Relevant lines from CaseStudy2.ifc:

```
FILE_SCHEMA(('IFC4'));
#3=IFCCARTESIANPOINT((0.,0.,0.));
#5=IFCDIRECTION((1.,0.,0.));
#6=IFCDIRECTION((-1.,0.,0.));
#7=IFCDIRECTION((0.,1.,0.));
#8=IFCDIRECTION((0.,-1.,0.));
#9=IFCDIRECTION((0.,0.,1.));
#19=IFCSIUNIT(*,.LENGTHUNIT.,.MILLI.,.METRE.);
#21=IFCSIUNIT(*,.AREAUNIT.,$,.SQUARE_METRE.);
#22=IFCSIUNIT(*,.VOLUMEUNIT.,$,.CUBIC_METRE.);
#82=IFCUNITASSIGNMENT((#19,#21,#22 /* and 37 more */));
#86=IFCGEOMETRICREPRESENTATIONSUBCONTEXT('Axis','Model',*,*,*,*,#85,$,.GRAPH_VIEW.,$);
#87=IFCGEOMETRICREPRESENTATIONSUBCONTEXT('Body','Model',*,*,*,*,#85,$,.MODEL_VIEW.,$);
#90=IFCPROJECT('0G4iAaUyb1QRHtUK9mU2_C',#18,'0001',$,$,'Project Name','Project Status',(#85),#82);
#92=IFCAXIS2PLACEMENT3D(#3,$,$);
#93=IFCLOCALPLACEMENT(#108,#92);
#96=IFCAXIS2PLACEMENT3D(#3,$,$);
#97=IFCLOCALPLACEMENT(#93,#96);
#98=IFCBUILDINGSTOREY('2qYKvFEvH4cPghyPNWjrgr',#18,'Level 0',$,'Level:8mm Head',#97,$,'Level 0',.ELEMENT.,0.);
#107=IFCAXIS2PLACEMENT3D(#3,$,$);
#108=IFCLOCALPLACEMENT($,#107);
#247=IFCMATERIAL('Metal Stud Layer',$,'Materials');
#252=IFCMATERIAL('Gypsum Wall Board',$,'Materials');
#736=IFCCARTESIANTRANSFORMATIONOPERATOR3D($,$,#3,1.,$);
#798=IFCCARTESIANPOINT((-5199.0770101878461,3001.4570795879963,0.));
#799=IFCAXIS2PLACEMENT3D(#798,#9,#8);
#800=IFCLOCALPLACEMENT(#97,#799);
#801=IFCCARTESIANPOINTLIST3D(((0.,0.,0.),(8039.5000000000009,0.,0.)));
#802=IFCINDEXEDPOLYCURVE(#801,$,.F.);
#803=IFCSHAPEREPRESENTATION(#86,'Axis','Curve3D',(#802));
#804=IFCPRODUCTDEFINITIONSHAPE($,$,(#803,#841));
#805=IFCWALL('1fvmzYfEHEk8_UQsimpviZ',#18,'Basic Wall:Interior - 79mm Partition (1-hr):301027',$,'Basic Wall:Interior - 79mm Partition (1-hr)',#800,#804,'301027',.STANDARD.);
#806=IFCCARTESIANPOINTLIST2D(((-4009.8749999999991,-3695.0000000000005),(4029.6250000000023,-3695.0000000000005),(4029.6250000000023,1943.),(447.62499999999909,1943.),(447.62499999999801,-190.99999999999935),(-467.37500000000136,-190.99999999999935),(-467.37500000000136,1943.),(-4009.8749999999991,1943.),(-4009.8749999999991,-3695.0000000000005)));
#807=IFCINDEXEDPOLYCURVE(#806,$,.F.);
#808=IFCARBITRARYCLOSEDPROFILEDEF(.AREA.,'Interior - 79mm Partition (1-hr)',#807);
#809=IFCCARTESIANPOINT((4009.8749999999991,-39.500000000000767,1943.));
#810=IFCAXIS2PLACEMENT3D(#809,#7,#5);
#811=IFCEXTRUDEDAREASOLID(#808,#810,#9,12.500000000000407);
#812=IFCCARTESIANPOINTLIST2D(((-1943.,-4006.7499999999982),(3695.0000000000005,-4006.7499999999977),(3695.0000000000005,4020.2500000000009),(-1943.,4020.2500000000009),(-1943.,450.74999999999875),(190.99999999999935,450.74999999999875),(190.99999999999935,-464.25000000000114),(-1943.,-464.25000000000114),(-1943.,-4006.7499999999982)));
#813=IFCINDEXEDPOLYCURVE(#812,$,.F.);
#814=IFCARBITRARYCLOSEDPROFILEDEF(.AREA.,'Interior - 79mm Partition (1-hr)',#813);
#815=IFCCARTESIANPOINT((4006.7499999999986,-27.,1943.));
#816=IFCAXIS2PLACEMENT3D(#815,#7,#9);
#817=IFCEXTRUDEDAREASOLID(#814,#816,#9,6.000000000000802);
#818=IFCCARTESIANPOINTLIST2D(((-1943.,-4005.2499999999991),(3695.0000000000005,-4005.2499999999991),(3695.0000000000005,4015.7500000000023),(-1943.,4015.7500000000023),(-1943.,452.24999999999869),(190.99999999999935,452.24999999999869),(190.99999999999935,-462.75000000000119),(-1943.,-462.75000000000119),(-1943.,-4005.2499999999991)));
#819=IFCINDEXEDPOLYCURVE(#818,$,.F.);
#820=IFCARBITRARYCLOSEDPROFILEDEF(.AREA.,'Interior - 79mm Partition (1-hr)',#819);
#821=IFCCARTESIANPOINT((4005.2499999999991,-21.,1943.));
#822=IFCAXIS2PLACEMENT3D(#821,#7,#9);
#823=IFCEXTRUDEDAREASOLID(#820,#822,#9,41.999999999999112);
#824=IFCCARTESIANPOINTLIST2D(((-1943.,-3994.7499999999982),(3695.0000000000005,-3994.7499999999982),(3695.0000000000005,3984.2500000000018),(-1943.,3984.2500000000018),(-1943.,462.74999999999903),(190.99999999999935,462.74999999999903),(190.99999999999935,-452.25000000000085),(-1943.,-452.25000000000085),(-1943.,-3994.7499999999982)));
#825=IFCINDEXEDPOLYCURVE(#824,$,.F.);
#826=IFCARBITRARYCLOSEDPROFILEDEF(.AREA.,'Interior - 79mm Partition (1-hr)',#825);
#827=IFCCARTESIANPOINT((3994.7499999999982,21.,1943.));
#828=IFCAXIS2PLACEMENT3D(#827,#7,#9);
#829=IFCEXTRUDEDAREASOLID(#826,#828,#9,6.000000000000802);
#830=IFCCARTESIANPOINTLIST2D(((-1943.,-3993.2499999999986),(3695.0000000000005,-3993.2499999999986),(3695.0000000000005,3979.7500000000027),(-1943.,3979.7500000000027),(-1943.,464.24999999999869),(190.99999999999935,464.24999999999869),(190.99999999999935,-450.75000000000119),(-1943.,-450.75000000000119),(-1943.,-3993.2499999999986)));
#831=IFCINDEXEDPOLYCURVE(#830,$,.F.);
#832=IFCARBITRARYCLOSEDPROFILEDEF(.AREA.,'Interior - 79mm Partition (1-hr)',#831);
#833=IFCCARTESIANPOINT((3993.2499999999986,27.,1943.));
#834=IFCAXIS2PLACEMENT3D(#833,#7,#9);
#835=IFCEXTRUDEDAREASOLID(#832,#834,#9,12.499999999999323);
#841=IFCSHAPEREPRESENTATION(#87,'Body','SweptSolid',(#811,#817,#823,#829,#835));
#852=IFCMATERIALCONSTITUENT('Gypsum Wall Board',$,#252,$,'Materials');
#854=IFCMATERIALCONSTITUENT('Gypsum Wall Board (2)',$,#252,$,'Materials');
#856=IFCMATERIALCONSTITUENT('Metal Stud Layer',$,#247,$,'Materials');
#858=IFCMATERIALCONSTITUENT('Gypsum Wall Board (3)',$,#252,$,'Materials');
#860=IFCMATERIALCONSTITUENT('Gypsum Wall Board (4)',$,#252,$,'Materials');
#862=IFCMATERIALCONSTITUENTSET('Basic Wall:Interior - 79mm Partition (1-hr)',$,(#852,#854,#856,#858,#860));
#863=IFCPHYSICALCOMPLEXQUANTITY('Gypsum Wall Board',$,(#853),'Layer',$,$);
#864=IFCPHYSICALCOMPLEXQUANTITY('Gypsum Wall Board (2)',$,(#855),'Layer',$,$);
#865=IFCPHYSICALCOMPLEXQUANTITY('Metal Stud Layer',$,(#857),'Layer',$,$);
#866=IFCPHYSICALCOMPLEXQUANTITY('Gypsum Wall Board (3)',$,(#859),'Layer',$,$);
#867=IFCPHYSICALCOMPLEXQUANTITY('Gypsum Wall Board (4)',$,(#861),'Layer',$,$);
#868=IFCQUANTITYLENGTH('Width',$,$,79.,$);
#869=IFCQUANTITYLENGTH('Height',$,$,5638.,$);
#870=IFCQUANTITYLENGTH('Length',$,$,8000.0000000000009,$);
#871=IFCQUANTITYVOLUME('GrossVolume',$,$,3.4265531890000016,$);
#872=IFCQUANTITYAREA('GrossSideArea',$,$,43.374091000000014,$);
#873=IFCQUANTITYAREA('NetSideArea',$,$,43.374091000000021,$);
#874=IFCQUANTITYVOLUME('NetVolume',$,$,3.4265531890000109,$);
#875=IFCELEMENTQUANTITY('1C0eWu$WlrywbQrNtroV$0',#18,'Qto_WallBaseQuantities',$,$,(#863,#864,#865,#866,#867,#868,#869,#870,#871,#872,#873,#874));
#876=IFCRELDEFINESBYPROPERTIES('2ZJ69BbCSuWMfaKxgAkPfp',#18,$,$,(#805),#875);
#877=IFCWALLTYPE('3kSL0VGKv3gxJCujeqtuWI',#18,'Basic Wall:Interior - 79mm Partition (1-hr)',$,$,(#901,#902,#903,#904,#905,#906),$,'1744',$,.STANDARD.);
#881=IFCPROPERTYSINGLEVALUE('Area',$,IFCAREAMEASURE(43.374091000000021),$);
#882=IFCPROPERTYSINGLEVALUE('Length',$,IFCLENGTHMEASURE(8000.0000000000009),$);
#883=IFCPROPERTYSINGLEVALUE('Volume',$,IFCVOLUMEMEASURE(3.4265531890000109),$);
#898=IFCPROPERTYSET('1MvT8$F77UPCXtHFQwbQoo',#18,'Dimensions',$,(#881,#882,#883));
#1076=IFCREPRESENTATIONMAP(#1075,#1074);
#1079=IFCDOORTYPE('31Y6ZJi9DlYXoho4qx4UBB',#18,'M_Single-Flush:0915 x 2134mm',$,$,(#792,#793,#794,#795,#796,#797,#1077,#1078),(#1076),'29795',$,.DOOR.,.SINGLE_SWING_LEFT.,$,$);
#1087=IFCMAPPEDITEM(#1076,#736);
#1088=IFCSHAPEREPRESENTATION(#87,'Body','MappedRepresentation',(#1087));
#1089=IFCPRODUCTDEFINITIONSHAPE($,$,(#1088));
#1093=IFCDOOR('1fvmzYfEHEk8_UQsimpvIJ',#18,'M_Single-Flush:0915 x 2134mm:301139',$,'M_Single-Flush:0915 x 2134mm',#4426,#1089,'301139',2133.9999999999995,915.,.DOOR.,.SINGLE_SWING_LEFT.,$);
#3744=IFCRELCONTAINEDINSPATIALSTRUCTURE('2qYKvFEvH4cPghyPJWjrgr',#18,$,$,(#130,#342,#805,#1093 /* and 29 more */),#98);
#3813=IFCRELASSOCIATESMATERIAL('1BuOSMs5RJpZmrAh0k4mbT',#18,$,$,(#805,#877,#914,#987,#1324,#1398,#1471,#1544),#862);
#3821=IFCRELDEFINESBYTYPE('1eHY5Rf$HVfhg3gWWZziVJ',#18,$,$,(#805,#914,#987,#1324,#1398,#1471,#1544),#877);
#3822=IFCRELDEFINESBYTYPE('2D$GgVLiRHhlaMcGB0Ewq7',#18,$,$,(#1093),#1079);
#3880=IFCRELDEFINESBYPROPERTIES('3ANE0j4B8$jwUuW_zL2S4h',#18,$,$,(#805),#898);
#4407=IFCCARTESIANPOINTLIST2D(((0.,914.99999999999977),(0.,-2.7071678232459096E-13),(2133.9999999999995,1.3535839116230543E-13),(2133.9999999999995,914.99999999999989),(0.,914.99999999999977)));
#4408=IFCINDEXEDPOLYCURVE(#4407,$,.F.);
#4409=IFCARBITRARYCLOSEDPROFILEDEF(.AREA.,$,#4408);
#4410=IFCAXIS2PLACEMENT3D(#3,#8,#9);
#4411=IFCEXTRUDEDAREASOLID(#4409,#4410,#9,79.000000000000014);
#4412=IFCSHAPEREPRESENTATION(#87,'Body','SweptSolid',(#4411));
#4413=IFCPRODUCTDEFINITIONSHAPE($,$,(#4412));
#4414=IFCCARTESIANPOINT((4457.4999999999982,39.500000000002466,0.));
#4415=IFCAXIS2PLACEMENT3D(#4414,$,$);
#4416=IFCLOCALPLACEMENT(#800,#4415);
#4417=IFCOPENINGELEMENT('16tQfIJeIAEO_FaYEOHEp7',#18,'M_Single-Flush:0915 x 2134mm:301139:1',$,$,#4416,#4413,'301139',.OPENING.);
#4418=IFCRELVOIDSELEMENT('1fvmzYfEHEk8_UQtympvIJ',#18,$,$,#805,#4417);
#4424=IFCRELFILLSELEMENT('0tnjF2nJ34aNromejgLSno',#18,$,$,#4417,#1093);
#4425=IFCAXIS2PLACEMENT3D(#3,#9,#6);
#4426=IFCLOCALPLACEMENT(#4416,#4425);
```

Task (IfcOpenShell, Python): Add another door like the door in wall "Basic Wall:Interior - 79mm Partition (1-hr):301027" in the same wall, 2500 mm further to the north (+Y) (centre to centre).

```python
import ifcopenshell
import ifcopenshell.api.feature
import ifcopenshell.api.geometry
import ifcopenshell.api.pset
import ifcopenshell.api.root
import ifcopenshell.geom
import ifcopenshell.util.element
import ifcopenshell.util.placement
import ifcopenshell.util.shape
import ifcopenshell.util.unit

model = ifcopenshell.open("CaseStudy2.ifc")
area_scale = ifcopenshell.util.unit.calculate_unit_scale(model, "AREAUNIT")
volume_scale = ifcopenshell.util.unit.calculate_unit_scale(model, "VOLUMEUNIT")
settings = ifcopenshell.geom.settings()


def volume(element):
    """Net volume in cubic metres, openings subtracted."""
    shape = ifcopenshell.geom.create_shape(settings, element)
    return ifcopenshell.util.shape.get_volume(shape.geometry)


def reuse_history(source, copy):
    """copy_class also copies each property set's owner history, people and application; keep the originals."""
    for rel in copy.IsDefinedBy:
        if rel.is_a("IfcRelDefinesByProperties") and (history := rel.RelatingPropertyDefinition.OwnerHistory):
            rel.RelatingPropertyDefinition.OwnerHistory = source.OwnerHistory
            ifcopenshell.util.element.remove_deep2(model, history)


door = model.by_guid("1fvmzYfEHEk8_UQsimpvIJ")
opening = door.FillsVoids[0].RelatingOpeningElement
wall = opening.VoidsElements[0].RelatingBuildingElement
before = volume(wall)
shift = ifcopenshell.util.placement.get_local_placement(wall.ObjectPlacement)[:3, 0] * -2500.0

# copy_class copies the void relationship, type, container and properties, but no geometry.
new_opening = ifcopenshell.api.root.copy_class(model, product=opening)
new_opening.Representation = ifcopenshell.util.element.copy_deep(
    model, opening.Representation, exclude=["IfcGeometricRepresentationContext", "IfcRepresentationMap"]
)
new_opening.Name = "M_Single-Flush:0915 x 2134mm"
new_opening.Tag = None
reuse_history(opening, new_opening)
new_door = ifcopenshell.api.root.copy_class(model, product=door)
new_door.Representation = ifcopenshell.util.element.copy_deep(
    model, door.Representation, exclude=["IfcGeometricRepresentationContext", "IfcRepresentationMap"]
)
new_door.Name = "M_Single-Flush:0915 x 2134mm"
new_door.Tag = None
reuse_history(door, new_door)
ifcopenshell.api.feature.add_filling(model, opening=new_opening, element=new_door)

for old, new in ((opening, new_opening), (door, new_door)):
    matrix = ifcopenshell.util.placement.get_local_placement(old.ObjectPlacement)
    matrix[:3, 3] += shift
    ifcopenshell.api.geometry.edit_object_placement(model, product=new, matrix=matrix, is_si=False)

after = volume(wall)
thickness = 0.079  # wall thickness in metres

# Update the wall's stored quantities.
qto = model.by_id(ifcopenshell.util.element.get_pset(wall, "Qto_WallBaseQuantities", should_inherit=False)["id"])
ifcopenshell.api.pset.edit_qto(model, qto=qto, properties={
    "NetSideArea": after / thickness / area_scale,
    "NetVolume": after / volume_scale,
})
pset = model.by_id(ifcopenshell.util.element.get_pset(wall, "Dimensions", should_inherit=False)["id"])
ifcopenshell.api.pset.edit_pset(model, pset=pset, properties={
    "Area": model.create_entity("IfcAreaMeasure", after / thickness / area_scale),
    "Volume": model.create_entity("IfcVolumeMeasure", after / volume_scale),
})

print(f"wall volume {before:.3f} -> {after:.3f} m3")

model.write("CaseStudy2-out.ifc")
```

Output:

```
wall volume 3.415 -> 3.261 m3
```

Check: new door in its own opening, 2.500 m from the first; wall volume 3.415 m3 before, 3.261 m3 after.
